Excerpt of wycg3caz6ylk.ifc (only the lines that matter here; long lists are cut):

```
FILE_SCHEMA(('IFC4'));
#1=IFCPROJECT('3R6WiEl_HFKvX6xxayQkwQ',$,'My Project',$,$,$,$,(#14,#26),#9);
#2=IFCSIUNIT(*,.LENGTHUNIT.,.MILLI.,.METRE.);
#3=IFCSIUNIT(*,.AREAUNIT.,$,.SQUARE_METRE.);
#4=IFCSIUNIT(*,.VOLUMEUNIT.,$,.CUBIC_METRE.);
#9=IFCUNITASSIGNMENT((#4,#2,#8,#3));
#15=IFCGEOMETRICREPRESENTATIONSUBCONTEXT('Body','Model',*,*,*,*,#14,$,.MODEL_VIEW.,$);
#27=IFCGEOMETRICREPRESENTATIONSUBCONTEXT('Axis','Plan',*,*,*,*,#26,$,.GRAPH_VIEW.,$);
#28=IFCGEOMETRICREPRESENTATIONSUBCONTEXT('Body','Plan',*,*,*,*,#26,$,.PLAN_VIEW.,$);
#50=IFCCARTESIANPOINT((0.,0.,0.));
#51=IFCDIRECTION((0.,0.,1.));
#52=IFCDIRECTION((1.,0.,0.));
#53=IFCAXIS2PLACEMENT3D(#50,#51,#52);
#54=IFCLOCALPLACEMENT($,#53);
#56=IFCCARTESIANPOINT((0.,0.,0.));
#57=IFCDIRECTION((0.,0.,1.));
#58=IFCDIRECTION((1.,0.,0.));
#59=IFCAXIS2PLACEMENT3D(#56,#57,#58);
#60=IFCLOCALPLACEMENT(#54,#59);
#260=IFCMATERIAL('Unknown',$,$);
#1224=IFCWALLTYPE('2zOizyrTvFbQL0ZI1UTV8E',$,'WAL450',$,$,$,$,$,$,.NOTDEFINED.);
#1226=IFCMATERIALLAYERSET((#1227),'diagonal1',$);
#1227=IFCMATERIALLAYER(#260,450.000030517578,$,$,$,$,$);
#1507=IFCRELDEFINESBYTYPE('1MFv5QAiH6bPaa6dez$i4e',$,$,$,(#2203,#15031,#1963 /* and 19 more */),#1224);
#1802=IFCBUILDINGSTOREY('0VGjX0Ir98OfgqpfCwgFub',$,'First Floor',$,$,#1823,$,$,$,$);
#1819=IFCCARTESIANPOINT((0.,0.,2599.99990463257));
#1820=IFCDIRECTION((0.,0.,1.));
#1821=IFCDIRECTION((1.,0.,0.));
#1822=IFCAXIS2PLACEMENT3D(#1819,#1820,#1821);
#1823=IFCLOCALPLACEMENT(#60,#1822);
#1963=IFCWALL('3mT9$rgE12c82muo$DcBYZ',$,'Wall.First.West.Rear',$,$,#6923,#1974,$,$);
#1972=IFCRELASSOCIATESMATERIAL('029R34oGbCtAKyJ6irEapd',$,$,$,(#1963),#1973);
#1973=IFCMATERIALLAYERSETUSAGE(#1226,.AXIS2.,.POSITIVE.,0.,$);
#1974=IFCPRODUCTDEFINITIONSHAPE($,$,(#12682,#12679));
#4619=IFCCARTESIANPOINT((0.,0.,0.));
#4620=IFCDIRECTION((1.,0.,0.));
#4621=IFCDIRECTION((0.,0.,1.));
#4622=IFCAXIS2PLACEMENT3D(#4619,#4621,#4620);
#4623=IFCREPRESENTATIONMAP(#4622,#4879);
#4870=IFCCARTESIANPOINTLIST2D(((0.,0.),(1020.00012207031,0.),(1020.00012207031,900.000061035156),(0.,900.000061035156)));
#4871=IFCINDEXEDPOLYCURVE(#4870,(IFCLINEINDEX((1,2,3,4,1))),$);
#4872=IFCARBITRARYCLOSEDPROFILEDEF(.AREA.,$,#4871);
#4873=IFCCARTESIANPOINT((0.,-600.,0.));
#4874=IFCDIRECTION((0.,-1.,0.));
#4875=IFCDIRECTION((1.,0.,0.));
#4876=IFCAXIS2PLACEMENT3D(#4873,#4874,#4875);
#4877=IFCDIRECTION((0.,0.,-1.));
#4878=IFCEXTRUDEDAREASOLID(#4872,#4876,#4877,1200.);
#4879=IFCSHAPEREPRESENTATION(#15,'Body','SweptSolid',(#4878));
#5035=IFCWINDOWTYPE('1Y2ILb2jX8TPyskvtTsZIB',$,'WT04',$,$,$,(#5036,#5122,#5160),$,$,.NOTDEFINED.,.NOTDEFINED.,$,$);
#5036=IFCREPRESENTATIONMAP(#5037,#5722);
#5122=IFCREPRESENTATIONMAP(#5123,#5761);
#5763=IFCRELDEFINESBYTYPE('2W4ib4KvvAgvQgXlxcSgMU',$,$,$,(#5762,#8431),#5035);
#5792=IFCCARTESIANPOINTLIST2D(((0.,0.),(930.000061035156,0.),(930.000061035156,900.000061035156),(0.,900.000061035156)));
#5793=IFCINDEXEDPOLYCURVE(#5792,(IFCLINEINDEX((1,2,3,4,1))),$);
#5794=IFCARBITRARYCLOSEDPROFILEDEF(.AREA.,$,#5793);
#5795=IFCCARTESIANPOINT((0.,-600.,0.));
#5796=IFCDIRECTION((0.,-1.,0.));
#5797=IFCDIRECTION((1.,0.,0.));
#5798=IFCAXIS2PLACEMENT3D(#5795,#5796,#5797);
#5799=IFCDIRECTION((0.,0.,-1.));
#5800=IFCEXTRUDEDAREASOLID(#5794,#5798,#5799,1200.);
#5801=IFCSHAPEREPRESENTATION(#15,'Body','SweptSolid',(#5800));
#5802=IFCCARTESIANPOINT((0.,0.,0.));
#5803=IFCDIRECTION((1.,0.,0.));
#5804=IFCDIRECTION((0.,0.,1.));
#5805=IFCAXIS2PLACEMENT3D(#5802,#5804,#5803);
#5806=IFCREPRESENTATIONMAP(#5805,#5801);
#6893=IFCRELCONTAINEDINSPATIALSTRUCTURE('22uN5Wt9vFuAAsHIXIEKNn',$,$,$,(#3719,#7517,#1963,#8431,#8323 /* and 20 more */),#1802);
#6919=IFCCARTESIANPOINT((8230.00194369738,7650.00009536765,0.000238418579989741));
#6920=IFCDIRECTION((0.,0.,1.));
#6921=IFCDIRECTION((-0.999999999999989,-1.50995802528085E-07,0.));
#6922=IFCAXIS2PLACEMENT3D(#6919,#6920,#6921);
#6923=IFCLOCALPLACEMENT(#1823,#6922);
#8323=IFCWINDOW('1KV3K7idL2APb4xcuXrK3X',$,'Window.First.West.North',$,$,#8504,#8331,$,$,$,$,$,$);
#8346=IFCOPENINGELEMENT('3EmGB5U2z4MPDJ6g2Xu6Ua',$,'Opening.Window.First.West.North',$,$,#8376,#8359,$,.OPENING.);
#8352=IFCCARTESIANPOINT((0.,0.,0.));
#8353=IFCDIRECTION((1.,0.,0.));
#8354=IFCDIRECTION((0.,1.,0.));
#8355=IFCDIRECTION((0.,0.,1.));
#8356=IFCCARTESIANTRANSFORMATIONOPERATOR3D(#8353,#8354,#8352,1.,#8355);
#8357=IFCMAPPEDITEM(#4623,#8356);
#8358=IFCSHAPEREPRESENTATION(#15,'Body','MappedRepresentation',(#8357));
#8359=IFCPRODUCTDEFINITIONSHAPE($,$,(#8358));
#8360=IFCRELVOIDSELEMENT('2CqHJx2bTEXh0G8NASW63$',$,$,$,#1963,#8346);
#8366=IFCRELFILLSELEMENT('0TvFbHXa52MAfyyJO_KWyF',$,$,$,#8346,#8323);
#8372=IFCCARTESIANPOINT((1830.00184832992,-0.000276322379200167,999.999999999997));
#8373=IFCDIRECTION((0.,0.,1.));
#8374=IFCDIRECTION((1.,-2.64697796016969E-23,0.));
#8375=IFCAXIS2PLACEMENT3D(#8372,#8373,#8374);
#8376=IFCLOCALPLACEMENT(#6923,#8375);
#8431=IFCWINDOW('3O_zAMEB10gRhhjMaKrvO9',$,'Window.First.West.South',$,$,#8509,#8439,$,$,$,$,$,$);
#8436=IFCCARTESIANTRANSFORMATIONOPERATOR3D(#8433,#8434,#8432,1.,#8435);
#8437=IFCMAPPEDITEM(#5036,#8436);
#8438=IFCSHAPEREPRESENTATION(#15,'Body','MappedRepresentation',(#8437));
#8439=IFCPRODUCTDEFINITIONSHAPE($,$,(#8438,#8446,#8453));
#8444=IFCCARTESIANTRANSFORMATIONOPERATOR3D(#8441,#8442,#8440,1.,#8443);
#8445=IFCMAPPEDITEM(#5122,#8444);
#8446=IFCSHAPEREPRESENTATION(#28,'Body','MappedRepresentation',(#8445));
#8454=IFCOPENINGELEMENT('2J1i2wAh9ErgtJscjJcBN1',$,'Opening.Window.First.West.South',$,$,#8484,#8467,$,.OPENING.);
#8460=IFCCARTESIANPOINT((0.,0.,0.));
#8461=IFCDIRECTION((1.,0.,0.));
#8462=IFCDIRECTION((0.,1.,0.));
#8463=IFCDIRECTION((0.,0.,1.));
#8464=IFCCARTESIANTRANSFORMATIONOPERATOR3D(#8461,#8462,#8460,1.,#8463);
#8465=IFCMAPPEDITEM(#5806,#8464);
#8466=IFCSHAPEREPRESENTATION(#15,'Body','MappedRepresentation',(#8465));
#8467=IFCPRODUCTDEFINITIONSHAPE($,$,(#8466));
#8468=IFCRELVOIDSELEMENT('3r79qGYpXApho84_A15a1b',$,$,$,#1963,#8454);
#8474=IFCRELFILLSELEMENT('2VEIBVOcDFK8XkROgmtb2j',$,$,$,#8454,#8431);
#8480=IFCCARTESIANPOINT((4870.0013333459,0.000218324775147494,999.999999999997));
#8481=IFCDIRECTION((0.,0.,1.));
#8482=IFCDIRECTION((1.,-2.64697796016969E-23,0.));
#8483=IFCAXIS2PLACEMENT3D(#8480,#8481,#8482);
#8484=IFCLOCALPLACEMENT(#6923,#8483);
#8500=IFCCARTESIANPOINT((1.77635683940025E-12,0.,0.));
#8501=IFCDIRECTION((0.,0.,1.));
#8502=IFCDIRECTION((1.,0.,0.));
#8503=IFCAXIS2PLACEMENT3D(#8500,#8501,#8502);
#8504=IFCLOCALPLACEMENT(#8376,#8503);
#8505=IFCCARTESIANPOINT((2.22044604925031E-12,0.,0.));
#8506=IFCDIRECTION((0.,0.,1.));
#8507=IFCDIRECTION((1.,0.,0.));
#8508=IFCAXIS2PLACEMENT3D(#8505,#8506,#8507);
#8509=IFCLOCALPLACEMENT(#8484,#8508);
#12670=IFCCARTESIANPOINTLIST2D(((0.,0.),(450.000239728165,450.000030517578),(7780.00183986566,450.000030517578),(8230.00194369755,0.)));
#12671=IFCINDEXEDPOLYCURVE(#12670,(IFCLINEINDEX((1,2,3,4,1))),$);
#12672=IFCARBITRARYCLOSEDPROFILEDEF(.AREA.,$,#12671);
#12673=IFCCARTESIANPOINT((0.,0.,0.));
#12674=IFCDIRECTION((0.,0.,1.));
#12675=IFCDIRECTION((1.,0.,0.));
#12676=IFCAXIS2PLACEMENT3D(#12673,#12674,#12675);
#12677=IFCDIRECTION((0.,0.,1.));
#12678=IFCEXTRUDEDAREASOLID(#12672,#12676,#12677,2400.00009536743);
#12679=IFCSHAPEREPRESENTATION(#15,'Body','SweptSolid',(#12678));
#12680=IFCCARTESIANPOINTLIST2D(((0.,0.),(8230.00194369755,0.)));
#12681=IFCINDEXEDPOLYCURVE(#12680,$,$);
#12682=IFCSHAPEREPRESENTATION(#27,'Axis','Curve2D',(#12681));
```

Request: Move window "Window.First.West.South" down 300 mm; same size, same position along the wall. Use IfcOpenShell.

```python
import numpy as np
import ifcopenshell
import ifcopenshell.api.geometry
import ifcopenshell.util.placement
import ifcopenshell.util.unit

model = ifcopenshell.open("wycg3caz6ylk.ifc")
unit_scale = ifcopenshell.util.unit.calculate_unit_scale(model)

window = model.by_guid("3O_zAMEB10gRhhjMaKrvO9")
opening = window.FillsVoids[0].RelatingOpeningElement
dz = -300.0

shift = np.array([0.0, 0.0, dz])
# The window is placed relative to its opening, so it follows when the opening moves.
matrix = ifcopenshell.util.placement.get_local_placement(opening.ObjectPlacement)
matrix[:3, 3] += shift
ifcopenshell.api.geometry.edit_object_placement(
    model, product=opening, matrix=matrix, is_si=False, should_transform_children=True
)

print(f"moved by {dz * unit_scale:+.3f} m")

model.write("wycg3caz6ylk_v2.ifc")
```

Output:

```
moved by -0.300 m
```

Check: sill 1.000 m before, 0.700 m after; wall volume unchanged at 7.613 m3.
